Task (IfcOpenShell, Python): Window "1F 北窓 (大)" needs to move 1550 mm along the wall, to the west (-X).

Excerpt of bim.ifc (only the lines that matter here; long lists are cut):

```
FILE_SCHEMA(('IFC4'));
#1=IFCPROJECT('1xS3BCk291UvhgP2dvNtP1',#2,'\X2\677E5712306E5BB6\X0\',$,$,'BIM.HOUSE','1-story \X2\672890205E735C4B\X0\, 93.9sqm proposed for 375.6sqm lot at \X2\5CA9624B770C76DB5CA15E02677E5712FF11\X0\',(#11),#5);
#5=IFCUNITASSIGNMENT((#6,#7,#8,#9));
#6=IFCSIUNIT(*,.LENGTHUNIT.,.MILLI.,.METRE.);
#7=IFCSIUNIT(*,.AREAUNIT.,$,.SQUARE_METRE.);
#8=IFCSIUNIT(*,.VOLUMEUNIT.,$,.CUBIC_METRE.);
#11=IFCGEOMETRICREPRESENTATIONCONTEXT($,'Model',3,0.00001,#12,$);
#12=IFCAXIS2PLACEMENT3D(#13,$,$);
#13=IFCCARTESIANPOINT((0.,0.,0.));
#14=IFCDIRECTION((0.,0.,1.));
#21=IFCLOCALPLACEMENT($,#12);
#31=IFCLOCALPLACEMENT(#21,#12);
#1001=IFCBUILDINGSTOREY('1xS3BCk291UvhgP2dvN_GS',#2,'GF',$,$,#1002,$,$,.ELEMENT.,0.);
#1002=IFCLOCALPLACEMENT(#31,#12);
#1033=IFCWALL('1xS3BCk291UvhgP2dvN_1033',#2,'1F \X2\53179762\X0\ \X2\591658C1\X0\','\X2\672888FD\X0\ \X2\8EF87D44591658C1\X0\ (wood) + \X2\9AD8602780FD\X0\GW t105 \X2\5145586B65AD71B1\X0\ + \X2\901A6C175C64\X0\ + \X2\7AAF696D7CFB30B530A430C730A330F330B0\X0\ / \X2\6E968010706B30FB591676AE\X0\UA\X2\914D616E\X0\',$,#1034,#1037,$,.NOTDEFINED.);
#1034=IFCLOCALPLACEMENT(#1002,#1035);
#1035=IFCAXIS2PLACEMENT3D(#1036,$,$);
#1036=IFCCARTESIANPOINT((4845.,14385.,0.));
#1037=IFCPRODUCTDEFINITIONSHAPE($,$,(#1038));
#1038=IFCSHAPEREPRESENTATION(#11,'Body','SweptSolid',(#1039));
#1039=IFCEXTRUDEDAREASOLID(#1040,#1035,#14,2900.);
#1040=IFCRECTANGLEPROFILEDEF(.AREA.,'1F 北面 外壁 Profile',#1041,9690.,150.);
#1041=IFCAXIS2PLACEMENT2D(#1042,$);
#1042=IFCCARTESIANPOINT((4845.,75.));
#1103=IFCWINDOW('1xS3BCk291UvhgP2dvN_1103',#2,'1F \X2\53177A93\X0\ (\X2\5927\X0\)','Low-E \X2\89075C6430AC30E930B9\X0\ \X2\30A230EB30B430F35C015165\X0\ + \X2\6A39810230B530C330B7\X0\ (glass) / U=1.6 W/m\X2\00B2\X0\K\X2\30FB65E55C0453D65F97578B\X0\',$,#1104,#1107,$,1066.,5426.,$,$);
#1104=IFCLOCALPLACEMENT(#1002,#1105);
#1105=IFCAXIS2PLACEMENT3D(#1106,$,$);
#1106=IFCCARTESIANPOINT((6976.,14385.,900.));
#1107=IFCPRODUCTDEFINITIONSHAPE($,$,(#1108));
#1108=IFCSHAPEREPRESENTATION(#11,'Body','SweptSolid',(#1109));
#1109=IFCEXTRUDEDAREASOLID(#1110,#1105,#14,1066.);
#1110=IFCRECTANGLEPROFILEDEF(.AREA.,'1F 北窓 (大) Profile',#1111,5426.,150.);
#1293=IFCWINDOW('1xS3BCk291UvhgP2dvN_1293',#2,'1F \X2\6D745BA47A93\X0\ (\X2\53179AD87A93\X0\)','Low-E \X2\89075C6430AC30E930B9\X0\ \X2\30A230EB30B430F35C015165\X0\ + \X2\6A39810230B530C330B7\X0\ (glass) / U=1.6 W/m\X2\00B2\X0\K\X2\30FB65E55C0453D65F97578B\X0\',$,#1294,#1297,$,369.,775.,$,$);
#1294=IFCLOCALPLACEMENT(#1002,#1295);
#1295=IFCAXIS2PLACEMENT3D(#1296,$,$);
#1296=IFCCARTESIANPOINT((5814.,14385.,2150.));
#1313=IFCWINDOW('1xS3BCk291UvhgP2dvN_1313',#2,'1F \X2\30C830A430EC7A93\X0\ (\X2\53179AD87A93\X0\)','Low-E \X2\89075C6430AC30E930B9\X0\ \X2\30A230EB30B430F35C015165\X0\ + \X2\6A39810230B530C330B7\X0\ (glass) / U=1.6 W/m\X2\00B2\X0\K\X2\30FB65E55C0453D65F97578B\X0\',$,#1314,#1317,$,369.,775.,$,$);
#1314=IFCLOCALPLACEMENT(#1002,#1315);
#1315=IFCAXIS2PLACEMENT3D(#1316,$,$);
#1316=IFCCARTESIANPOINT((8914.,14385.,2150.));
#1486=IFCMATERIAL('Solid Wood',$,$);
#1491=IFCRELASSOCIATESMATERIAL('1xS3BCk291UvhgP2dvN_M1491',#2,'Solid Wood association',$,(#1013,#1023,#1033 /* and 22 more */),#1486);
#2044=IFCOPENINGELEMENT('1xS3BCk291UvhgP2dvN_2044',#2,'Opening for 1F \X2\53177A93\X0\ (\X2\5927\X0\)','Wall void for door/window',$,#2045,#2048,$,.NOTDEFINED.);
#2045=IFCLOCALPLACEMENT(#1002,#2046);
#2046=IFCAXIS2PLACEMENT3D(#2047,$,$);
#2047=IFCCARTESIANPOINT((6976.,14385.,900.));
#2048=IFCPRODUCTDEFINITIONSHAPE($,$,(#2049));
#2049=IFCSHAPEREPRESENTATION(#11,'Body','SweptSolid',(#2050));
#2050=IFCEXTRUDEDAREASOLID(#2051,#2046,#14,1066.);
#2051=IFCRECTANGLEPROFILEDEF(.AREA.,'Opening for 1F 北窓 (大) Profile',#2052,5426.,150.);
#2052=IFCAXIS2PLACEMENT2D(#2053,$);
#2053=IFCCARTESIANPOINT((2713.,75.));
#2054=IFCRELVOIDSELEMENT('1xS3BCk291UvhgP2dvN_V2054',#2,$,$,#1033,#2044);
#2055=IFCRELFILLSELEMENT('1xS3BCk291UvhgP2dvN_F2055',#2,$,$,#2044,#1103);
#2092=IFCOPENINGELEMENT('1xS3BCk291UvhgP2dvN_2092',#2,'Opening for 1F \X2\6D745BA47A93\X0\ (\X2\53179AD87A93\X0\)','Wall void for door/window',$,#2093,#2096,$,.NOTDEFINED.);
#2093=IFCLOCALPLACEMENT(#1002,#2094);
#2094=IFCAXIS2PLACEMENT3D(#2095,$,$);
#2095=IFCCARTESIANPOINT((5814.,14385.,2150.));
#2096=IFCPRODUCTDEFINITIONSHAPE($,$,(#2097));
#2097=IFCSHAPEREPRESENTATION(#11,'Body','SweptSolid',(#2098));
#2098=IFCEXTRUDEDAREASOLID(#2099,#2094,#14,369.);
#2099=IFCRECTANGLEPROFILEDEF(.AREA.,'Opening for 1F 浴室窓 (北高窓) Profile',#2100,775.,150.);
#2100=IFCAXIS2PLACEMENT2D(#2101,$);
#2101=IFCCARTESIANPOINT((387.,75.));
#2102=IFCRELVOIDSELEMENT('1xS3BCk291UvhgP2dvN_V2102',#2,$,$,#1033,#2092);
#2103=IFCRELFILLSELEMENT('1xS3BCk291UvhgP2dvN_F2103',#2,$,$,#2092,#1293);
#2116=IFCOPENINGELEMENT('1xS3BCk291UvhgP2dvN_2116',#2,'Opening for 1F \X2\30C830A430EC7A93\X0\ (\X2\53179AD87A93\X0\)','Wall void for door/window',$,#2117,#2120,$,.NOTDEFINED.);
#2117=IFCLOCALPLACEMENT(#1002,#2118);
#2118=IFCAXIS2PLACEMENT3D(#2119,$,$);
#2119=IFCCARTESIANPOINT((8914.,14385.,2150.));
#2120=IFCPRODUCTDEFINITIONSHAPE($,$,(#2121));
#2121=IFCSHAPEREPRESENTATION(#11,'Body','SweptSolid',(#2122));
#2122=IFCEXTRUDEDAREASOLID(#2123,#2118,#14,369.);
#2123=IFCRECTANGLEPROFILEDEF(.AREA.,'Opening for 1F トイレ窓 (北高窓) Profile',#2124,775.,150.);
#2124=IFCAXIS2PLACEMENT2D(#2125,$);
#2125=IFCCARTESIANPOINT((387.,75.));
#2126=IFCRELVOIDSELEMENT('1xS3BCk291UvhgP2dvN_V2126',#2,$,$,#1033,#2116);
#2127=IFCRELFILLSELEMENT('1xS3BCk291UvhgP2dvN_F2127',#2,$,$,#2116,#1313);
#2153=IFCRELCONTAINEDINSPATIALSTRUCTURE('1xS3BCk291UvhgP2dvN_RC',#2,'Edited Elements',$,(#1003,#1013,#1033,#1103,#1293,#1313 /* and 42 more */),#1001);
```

```python
import ifcopenshell
import ifcopenshell.api.geometry
import ifcopenshell.util.placement
import ifcopenshell.util.unit

model = ifcopenshell.open("bim.ifc")
unit_scale = ifcopenshell.util.unit.calculate_unit_scale(model)

window = model.by_guid("1xS3BCk291UvhgP2dvN_1103")
opening = window.FillsVoids[0].RelatingOpeningElement
wall = opening.VoidsElements[0].RelatingBuildingElement

wall_matrix = ifcopenshell.util.placement.get_local_placement(wall.ObjectPlacement)
shift = wall_matrix[:3, 0] * -1.55 / unit_scale
before = ifcopenshell.util.placement.get_local_placement(window.ObjectPlacement)[:3, 3].copy()

# The window is not placed relative to its opening, so move both.
for product in (opening, window):
    matrix = ifcopenshell.util.placement.get_local_placement(product.ObjectPlacement)
    matrix[:3, 3] += shift
    ifcopenshell.api.geometry.edit_object_placement(model, product=product, matrix=matrix, is_si=False)

after = ifcopenshell.util.placement.get_local_placement(window.ObjectPlacement)[:3, 3]
print("window moved by", (after - before).round(3) + 0.0)

model.write("bim-out.ifc")
```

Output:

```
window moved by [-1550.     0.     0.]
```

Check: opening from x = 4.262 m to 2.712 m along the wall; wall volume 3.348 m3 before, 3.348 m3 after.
